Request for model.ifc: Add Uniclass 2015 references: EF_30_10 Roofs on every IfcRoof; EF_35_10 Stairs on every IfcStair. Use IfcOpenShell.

First a look at what the model holds.

```python
import ifcopenshell

model = ifcopenshell.open("model.ifc")
print(model.schema)
print("classifications:", [c.Name for c in model.by_type("IfcClassification")])
for ifc_class in ("IfcDoor", "IfcRoof", "IfcStair", "IfcWall", "IfcWindow"):
    print(ifc_class, len(model.by_type(ifc_class)))
```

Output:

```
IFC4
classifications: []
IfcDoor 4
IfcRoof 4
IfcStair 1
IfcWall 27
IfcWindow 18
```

```python
import ifcopenshell
import ifcopenshell.api.classification

model = ifcopenshell.open("model.ifc")

system = ifcopenshell.api.classification.add_classification(model, classification="Uniclass 2015")

codes = {
    "IfcRoof": ("EF_30_10", "Roofs"),
    "IfcStair": ("EF_35_10", "Stairs"),
}
for ifc_class, (code, name) in codes.items():
    products = model.by_type(ifc_class)
    ifcopenshell.api.classification.add_reference(
        model, products=products, classification=system, identification=code, name=name
    )
    print(code, len(products))

model.write("model_rev.ifc")
```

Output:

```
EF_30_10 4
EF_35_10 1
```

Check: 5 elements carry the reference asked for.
